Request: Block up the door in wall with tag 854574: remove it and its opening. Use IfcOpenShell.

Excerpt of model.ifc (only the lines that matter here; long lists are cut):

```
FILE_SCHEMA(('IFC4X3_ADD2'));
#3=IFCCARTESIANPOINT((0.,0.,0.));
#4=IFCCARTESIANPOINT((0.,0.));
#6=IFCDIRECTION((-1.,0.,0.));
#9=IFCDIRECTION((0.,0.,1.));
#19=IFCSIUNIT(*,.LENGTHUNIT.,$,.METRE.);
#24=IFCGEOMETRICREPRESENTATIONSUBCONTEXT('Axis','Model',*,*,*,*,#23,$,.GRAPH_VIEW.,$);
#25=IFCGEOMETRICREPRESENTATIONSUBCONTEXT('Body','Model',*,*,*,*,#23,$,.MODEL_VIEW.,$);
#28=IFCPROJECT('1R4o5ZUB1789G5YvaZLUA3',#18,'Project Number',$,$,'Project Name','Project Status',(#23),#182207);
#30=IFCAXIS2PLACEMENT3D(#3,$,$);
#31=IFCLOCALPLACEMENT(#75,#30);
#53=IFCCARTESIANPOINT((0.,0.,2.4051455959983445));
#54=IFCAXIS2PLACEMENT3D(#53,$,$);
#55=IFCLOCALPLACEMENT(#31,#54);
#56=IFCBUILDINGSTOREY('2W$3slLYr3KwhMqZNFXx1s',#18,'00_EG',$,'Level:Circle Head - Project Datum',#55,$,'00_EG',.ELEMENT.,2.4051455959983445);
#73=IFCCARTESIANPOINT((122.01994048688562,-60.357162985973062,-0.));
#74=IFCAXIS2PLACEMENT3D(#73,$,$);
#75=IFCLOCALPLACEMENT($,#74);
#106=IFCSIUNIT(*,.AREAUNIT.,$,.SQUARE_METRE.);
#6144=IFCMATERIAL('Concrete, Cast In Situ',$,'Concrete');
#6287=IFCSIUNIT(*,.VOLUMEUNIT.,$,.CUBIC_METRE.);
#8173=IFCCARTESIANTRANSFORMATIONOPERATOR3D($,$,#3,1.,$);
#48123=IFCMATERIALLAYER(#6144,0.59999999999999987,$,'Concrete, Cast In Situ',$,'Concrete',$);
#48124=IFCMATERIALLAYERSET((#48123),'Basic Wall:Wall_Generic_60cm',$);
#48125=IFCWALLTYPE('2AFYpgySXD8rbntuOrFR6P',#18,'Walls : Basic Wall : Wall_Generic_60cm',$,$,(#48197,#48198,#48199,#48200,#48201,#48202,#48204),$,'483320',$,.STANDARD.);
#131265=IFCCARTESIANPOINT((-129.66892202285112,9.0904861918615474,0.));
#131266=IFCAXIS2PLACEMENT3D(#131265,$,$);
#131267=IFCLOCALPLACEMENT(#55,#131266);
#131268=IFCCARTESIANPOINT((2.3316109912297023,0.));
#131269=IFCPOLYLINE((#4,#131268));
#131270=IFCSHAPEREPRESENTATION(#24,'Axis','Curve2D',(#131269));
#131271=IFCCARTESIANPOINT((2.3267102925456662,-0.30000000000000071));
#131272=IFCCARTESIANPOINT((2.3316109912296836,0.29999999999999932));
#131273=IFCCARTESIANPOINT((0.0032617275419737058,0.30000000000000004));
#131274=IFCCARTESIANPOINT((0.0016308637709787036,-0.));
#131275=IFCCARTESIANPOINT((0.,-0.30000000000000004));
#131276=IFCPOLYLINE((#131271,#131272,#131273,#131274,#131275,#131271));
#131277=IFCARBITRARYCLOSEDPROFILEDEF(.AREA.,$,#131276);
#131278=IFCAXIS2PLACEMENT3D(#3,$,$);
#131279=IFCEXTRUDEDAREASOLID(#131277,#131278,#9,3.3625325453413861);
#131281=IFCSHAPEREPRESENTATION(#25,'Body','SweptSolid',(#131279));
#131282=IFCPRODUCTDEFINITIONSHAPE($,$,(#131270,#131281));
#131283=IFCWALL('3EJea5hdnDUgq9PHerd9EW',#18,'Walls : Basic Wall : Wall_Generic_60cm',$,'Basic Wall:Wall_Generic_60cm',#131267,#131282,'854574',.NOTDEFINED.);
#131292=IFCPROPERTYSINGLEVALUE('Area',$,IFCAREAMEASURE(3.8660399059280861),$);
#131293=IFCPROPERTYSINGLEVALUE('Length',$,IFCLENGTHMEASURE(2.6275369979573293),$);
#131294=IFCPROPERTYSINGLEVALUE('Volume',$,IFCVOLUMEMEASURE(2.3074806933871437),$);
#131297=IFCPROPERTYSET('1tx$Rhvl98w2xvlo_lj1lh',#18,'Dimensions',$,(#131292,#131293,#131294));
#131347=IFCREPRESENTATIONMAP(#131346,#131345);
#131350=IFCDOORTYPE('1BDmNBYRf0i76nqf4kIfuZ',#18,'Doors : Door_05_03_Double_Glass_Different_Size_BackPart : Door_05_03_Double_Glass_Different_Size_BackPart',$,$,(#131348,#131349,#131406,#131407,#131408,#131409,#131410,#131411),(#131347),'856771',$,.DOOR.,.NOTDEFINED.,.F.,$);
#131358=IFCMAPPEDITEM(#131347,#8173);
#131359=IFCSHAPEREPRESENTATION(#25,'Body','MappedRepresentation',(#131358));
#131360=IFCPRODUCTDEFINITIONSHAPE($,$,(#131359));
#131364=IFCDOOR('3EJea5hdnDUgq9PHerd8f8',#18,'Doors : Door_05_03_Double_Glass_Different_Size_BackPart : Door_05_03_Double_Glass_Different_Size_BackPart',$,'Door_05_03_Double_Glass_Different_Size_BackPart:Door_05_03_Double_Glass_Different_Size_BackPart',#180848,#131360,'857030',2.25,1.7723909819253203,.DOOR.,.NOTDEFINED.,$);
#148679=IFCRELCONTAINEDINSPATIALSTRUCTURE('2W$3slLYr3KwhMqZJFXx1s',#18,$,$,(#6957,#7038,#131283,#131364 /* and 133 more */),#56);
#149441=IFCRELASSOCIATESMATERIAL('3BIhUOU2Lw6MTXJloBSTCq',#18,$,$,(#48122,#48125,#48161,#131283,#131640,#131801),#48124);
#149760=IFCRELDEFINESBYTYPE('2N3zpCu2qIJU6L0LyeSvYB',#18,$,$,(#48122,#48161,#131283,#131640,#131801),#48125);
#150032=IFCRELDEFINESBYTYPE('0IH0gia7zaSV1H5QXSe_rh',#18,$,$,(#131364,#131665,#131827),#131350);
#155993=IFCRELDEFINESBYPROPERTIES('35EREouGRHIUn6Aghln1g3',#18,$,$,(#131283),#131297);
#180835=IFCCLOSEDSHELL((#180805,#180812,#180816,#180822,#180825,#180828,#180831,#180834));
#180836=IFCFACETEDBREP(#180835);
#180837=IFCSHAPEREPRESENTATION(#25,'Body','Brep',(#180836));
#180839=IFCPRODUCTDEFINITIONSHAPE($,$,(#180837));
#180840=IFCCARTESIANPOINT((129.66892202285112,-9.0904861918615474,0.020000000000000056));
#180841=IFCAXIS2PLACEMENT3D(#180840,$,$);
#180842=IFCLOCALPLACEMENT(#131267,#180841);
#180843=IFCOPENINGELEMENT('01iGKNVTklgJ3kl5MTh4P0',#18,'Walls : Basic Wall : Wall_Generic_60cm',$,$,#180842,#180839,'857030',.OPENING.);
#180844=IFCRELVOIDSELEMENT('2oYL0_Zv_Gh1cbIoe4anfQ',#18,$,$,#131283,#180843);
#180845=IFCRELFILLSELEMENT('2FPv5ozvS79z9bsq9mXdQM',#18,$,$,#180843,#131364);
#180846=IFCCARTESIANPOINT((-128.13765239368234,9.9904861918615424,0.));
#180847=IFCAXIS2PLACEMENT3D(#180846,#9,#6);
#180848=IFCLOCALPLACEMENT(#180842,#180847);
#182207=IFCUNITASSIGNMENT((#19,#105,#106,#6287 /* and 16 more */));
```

```python
import ifcopenshell
import ifcopenshell.api.feature
import ifcopenshell.api.pset
import ifcopenshell.api.root
import ifcopenshell.geom
import ifcopenshell.util.element
import ifcopenshell.util.shape
import ifcopenshell.util.unit

model = ifcopenshell.open("model.ifc")
area_scale = ifcopenshell.util.unit.calculate_unit_scale(model, "AREAUNIT")
volume_scale = ifcopenshell.util.unit.calculate_unit_scale(model, "VOLUMEUNIT")
settings = ifcopenshell.geom.settings()


def volume(element):
    """Net volume in cubic metres, openings subtracted."""
    shape = ifcopenshell.geom.create_shape(settings, element)
    return ifcopenshell.util.shape.get_volume(shape.geometry)


door = model.by_id(131364)
opening = door.FillsVoids[0].RelatingOpeningElement
wall = opening.VoidsElements[0].RelatingBuildingElement
before = volume(wall)

ifcopenshell.api.root.remove_product(model, product=door)
ifcopenshell.api.feature.remove_feature(model, feature=opening)

after = volume(wall)
thickness = 0.6  # wall thickness in metres

# Update the wall's stored quantities.
pset = model.by_id(ifcopenshell.util.element.get_pset(wall, "Dimensions", should_inherit=False)["id"])
ifcopenshell.api.pset.edit_pset(model, pset=pset, properties={
    "Area": model.create_entity("IfcAreaMeasure", after / thickness / area_scale),
    "Volume": model.create_entity("IfcVolumeMeasure", after / volume_scale),
})

print(f"wall volume {before:.3f} -> {after:.3f} m3")

model.write("model_rev.ifc")
```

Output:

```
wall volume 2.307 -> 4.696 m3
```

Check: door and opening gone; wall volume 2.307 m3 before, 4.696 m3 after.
